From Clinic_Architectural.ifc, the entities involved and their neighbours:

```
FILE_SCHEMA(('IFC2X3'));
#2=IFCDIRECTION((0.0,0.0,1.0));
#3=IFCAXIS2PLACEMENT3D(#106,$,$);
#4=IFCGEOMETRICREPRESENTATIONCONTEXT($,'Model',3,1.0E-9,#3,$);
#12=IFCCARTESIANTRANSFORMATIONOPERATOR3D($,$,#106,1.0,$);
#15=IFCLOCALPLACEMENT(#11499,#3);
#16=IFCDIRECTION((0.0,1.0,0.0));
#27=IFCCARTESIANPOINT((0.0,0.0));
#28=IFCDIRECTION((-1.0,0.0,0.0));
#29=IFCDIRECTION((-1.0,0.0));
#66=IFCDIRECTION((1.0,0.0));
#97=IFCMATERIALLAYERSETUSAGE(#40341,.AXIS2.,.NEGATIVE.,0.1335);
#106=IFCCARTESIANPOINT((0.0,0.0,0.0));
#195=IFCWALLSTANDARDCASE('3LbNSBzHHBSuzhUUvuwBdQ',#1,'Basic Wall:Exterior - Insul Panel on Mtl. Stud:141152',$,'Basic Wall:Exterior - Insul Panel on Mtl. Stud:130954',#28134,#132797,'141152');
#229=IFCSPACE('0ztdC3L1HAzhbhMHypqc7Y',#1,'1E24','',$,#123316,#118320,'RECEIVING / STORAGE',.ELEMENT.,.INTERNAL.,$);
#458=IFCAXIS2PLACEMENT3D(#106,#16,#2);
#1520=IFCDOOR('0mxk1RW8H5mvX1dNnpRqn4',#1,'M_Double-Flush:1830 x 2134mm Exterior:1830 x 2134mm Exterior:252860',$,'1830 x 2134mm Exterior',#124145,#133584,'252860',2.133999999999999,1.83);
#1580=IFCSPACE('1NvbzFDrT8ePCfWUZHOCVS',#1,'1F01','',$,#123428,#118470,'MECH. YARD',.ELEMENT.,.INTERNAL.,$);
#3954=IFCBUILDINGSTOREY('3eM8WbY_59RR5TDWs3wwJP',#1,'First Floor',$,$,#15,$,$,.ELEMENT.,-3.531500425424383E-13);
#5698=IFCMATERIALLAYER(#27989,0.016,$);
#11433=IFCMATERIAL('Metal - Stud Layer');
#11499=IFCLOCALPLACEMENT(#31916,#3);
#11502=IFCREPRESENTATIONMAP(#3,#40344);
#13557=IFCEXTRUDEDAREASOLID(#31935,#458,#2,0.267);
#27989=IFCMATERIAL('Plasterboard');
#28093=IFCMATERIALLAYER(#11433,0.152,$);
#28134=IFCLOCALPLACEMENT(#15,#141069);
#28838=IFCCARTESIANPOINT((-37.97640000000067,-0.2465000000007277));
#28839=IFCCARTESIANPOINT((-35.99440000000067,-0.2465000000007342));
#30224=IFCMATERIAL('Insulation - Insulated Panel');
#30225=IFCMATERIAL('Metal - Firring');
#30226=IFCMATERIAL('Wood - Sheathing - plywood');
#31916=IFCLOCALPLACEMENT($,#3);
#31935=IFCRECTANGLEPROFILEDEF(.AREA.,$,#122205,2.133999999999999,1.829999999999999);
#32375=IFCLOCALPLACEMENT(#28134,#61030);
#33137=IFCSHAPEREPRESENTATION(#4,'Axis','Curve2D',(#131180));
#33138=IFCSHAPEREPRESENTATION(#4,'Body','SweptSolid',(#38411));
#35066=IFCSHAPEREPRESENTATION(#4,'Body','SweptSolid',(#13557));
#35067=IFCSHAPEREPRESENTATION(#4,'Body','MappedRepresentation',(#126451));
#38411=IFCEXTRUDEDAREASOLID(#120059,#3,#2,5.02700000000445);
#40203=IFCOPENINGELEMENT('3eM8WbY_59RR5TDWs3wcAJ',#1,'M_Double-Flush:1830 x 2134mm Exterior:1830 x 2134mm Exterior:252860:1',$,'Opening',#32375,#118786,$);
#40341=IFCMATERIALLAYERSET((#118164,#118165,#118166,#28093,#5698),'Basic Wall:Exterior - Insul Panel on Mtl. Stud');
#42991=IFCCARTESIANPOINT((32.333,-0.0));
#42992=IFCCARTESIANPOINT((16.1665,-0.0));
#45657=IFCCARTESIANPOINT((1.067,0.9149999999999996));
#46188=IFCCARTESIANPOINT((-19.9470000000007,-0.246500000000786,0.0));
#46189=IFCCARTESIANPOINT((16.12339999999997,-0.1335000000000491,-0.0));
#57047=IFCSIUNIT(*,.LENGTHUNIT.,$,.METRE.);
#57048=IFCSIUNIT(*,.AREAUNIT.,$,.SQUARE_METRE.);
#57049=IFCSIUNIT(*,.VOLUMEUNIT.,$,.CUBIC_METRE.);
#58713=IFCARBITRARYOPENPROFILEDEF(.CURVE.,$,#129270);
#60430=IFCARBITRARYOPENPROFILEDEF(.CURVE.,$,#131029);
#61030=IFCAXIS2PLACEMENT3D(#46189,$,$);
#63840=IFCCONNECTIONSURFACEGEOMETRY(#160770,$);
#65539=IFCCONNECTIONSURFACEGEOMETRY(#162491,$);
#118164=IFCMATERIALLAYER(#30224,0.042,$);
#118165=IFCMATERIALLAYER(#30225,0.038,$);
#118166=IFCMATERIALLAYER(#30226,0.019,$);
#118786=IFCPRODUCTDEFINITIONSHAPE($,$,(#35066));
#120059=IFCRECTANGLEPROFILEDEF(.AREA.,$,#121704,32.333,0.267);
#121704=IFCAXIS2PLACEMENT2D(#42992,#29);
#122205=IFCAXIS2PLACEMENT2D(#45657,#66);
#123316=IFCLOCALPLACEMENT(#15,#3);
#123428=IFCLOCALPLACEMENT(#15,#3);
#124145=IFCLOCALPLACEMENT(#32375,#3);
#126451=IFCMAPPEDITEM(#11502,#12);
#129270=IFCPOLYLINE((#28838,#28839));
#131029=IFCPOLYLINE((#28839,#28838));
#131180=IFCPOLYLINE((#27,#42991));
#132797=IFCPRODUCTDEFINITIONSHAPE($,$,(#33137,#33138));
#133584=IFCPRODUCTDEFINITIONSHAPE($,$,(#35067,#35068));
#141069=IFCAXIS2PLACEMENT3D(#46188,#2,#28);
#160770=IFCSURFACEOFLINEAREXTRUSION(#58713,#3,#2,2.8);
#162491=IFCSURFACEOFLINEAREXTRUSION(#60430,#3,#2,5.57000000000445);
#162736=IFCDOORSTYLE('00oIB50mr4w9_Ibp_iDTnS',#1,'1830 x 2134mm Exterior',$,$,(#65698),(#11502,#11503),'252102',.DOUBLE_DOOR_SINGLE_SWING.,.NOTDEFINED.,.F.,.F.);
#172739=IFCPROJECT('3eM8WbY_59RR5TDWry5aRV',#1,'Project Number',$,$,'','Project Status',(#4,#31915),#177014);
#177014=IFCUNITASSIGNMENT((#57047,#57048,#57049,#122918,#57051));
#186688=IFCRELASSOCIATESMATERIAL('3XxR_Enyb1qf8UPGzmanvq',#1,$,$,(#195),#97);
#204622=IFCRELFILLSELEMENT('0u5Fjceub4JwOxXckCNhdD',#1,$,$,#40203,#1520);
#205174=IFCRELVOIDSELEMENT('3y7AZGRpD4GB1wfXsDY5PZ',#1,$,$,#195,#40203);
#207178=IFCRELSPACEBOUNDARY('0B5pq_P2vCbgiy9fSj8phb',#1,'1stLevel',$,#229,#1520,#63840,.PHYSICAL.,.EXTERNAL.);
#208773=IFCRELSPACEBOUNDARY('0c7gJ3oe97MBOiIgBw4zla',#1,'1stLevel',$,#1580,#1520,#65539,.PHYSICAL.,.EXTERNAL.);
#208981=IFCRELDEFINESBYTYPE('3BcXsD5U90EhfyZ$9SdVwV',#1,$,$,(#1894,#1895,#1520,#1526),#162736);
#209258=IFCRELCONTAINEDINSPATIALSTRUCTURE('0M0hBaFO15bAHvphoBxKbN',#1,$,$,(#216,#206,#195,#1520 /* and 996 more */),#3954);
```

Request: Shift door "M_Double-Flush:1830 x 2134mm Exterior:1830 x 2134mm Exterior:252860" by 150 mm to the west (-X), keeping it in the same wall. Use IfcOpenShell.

```python
import numpy as np
import ifcopenshell
import ifcopenshell.api.geometry
import ifcopenshell.util.placement
import ifcopenshell.util.unit

model = ifcopenshell.open("Clinic_Architectural.ifc")
unit_scale = ifcopenshell.util.unit.calculate_unit_scale(model)

door = model.by_guid("0mxk1RW8H5mvX1dNnpRqn4")
opening = door.FillsVoids[0].RelatingOpeningElement
wall = opening.VoidsElements[0].RelatingBuildingElement

wall_matrix = ifcopenshell.util.placement.get_local_placement(wall.ObjectPlacement)
shift = wall_matrix[:3, 0] * 0.15 / unit_scale
before = ifcopenshell.util.placement.get_local_placement(door.ObjectPlacement)[:3, 3].copy()

# The door is placed relative to its opening, so it follows when the opening moves.
matrix = ifcopenshell.util.placement.get_local_placement(opening.ObjectPlacement)
matrix[:3, 3] += shift
ifcopenshell.api.geometry.edit_object_placement(
    model, product=opening, matrix=matrix, is_si=False, should_transform_children=True
)

# Space boundary surfaces are stored in each space's coordinates; move them too.
for rel in door.ProvidesBoundaries:
    if not rel.ConnectionGeometry:
        continue
    surface = rel.ConnectionGeometry.SurfaceOnRelatingElement
    space_matrix = ifcopenshell.util.placement.get_local_placement(rel.RelatingSpace.ObjectPlacement)
    point = np.array(surface.Position.Location.Coordinates) + space_matrix[:3, :3].T @ shift
    surface.Position = model.createIfcAxis2Placement3D(
        model.createIfcCartesianPoint(point.tolist()), surface.Position.Axis, surface.Position.RefDirection
    )

after = ifcopenshell.util.placement.get_local_placement(door.ObjectPlacement)[:3, 3]
print("door moved by", (after - before).round(3) + 0.0)

model.write("Clinic_Architectural_rev.ifc")
```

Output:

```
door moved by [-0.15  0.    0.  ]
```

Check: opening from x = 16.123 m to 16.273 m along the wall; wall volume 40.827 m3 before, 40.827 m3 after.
